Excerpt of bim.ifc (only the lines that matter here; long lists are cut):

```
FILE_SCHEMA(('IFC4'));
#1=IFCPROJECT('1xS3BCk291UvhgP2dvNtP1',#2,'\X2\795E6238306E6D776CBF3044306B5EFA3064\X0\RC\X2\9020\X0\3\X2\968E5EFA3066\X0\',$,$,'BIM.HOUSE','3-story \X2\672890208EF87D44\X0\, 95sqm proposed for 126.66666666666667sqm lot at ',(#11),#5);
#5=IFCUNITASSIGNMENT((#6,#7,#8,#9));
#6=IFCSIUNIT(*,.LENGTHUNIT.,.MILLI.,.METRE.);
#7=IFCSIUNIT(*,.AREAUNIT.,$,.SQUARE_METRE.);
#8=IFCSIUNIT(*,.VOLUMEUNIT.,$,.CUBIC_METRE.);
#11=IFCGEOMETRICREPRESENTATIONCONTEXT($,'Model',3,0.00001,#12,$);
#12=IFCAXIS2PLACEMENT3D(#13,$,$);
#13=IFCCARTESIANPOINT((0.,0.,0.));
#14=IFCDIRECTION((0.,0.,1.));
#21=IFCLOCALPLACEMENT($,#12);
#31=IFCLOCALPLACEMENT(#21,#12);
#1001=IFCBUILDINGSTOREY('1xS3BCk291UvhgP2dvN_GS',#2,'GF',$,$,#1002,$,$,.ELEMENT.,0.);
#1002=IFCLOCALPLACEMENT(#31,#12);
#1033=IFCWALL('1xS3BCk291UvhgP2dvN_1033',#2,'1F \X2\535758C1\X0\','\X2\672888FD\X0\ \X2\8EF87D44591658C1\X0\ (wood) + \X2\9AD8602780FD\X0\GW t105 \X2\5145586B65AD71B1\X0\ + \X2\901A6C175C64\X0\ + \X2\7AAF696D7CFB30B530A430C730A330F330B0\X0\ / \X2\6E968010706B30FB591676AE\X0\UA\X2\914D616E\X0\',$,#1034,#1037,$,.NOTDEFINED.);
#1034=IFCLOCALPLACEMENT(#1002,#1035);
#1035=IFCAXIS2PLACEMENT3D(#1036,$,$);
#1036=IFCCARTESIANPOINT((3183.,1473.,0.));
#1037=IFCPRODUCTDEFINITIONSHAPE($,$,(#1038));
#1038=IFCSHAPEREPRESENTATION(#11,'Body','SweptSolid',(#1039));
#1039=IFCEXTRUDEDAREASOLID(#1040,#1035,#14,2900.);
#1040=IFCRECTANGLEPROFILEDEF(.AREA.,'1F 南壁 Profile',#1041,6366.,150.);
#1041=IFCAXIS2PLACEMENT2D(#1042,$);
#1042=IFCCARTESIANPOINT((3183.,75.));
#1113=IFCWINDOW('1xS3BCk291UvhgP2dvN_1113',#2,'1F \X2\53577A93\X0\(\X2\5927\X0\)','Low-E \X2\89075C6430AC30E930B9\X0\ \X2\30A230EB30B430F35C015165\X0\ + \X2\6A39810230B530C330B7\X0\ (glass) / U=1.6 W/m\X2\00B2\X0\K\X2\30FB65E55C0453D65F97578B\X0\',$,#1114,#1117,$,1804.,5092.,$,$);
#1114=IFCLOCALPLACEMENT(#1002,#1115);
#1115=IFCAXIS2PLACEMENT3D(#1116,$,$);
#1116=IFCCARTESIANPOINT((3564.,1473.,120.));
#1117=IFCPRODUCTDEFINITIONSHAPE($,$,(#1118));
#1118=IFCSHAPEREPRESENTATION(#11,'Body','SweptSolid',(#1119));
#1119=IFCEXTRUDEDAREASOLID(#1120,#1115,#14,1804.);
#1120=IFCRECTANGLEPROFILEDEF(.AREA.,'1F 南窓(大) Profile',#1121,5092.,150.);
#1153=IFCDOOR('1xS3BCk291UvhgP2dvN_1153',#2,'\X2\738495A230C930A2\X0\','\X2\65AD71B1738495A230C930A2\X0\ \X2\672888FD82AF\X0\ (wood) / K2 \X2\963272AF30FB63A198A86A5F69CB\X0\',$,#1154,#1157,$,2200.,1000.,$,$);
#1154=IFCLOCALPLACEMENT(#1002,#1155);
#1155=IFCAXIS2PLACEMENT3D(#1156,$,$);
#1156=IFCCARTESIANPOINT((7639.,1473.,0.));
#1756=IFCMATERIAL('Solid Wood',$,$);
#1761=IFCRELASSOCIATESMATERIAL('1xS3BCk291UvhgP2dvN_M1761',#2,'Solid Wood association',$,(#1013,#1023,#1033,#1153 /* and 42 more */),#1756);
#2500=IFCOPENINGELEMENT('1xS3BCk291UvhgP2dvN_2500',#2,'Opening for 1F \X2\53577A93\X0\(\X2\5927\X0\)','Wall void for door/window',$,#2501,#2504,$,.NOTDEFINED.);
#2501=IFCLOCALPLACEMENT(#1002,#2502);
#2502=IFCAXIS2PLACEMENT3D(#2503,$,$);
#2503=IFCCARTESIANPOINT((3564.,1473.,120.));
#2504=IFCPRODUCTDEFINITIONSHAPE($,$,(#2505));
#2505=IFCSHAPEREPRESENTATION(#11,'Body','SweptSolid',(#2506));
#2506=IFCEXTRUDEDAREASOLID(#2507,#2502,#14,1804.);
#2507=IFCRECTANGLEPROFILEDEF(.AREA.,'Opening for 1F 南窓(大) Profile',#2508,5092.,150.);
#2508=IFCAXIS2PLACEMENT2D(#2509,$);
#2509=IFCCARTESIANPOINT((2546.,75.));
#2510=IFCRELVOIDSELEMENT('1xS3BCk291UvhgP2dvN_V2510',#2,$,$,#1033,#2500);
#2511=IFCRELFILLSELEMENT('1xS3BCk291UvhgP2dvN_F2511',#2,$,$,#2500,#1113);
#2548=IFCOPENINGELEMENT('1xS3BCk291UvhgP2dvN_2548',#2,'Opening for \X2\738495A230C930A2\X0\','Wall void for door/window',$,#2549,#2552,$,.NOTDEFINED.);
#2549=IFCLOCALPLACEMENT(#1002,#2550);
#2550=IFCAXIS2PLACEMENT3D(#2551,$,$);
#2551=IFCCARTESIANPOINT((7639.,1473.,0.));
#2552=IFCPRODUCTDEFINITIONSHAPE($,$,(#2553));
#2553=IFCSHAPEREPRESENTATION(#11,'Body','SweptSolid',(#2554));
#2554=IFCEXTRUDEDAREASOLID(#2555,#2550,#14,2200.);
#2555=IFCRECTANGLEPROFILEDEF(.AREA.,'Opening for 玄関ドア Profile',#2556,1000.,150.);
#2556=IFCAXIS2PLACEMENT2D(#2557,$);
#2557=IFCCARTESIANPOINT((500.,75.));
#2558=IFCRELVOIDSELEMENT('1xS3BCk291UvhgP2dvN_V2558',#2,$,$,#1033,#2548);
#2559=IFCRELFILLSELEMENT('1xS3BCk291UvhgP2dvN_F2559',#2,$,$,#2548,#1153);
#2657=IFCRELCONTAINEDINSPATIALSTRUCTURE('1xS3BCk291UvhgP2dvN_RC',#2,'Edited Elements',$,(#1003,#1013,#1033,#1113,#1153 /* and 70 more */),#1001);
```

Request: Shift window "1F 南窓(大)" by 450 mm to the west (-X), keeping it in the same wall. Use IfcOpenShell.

```python
import ifcopenshell
import ifcopenshell.api.geometry
import ifcopenshell.util.placement
import ifcopenshell.util.unit

model = ifcopenshell.open("bim.ifc")
unit_scale = ifcopenshell.util.unit.calculate_unit_scale(model)

window = model.by_guid("1xS3BCk291UvhgP2dvN_1113")
opening = window.FillsVoids[0].RelatingOpeningElement
wall = opening.VoidsElements[0].RelatingBuildingElement

wall_matrix = ifcopenshell.util.placement.get_local_placement(wall.ObjectPlacement)
shift = wall_matrix[:3, 0] * -0.45 / unit_scale
before = ifcopenshell.util.placement.get_local_placement(window.ObjectPlacement)[:3, 3].copy()

# The window is not placed relative to its opening, so move both.
for product in (opening, window):
    matrix = ifcopenshell.util.placement.get_local_placement(product.ObjectPlacement)
    matrix[:3, 3] += shift
    ifcopenshell.api.geometry.edit_object_placement(model, product=product, matrix=matrix, is_si=False)

after = ifcopenshell.util.placement.get_local_placement(window.ObjectPlacement)[:3, 3]
print("window moved by", (after - before).round(3) + 0.0)

model.write("bim_v2.ifc")
```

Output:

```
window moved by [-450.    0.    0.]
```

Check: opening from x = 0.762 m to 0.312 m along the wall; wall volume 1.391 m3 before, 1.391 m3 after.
